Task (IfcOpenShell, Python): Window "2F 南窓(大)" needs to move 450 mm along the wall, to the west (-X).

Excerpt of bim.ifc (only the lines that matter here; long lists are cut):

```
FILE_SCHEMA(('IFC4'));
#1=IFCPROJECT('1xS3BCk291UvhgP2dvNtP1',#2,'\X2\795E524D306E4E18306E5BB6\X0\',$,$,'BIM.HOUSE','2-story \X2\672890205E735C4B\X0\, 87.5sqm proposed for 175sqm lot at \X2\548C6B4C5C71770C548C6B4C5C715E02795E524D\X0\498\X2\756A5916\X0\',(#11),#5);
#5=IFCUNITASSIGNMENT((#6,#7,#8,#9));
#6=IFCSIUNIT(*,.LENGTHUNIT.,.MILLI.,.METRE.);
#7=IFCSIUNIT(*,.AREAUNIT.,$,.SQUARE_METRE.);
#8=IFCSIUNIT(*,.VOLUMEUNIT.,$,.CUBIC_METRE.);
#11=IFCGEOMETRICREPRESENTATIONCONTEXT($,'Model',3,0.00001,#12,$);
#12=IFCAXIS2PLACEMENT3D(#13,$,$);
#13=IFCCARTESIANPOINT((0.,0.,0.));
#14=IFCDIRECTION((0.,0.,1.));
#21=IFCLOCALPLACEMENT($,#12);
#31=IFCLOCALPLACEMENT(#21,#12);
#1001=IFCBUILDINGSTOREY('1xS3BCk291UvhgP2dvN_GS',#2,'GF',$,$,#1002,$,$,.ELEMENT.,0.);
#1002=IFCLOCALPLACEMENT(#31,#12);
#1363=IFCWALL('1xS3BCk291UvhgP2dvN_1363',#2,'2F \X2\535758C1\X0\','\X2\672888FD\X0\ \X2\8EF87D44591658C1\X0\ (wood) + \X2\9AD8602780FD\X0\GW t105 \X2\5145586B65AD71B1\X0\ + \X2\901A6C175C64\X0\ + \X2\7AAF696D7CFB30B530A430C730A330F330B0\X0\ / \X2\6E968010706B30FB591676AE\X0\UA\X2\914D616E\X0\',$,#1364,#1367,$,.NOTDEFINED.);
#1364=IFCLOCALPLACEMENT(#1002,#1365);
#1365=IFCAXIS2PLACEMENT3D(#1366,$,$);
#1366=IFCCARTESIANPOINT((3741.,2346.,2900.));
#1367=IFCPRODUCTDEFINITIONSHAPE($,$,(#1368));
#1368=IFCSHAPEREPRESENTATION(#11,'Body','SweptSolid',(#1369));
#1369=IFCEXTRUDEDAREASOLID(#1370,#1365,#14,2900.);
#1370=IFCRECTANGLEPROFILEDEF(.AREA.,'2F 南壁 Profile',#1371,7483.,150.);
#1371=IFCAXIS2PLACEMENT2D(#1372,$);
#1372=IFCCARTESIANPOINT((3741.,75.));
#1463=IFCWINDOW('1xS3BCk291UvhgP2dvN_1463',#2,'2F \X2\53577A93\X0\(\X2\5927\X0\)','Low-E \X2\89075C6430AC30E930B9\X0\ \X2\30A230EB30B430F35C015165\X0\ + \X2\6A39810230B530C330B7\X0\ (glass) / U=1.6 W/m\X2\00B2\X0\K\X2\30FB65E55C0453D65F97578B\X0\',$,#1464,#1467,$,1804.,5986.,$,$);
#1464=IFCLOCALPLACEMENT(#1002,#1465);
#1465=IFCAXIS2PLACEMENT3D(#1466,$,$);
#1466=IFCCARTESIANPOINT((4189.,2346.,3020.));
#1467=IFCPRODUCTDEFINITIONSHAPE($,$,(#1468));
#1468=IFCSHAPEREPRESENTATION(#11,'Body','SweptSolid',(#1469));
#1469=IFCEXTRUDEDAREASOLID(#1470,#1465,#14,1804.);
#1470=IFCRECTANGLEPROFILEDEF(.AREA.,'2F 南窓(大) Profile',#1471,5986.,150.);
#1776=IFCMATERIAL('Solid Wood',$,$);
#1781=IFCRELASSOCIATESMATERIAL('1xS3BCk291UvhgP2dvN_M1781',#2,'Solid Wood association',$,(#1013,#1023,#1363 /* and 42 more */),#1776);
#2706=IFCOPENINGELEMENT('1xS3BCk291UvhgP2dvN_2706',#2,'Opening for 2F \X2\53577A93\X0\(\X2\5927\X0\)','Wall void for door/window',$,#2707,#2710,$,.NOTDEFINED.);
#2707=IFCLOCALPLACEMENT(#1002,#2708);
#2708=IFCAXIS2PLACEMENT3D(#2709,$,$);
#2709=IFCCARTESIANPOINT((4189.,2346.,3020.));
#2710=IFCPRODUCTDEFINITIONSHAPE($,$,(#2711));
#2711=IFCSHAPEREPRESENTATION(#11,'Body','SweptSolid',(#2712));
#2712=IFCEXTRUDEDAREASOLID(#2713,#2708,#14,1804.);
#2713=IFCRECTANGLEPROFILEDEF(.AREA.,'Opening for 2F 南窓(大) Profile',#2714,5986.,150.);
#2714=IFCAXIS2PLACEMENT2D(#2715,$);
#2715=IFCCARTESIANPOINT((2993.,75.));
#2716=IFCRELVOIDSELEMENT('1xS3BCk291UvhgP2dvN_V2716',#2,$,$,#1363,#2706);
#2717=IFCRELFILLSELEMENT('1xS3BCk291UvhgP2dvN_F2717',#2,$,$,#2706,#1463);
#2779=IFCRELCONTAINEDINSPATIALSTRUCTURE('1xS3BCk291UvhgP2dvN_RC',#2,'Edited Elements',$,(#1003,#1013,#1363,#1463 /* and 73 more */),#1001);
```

```python
import ifcopenshell
import ifcopenshell.api.geometry
import ifcopenshell.util.placement
import ifcopenshell.util.unit

model = ifcopenshell.open("bim.ifc")
unit_scale = ifcopenshell.util.unit.calculate_unit_scale(model)

window = model.by_guid("1xS3BCk291UvhgP2dvN_1463")
opening = window.FillsVoids[0].RelatingOpeningElement
wall = opening.VoidsElements[0].RelatingBuildingElement

wall_matrix = ifcopenshell.util.placement.get_local_placement(wall.ObjectPlacement)
shift = wall_matrix[:3, 0] * -0.45 / unit_scale
before = ifcopenshell.util.placement.get_local_placement(window.ObjectPlacement)[:3, 3].copy()

# The window is not placed relative to its opening, so move both.
for product in (opening, window):
    matrix = ifcopenshell.util.placement.get_local_placement(product.ObjectPlacement)
    matrix[:3, 3] += shift
    ifcopenshell.api.geometry.edit_object_placement(model, product=product, matrix=matrix, is_si=False)

after = ifcopenshell.util.placement.get_local_placement(window.ObjectPlacement)[:3, 3]
print("window moved by", (after - before).round(3) + 0.0)

model.write("bim_v2.ifc")
```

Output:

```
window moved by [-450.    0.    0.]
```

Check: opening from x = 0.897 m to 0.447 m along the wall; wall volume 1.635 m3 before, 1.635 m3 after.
